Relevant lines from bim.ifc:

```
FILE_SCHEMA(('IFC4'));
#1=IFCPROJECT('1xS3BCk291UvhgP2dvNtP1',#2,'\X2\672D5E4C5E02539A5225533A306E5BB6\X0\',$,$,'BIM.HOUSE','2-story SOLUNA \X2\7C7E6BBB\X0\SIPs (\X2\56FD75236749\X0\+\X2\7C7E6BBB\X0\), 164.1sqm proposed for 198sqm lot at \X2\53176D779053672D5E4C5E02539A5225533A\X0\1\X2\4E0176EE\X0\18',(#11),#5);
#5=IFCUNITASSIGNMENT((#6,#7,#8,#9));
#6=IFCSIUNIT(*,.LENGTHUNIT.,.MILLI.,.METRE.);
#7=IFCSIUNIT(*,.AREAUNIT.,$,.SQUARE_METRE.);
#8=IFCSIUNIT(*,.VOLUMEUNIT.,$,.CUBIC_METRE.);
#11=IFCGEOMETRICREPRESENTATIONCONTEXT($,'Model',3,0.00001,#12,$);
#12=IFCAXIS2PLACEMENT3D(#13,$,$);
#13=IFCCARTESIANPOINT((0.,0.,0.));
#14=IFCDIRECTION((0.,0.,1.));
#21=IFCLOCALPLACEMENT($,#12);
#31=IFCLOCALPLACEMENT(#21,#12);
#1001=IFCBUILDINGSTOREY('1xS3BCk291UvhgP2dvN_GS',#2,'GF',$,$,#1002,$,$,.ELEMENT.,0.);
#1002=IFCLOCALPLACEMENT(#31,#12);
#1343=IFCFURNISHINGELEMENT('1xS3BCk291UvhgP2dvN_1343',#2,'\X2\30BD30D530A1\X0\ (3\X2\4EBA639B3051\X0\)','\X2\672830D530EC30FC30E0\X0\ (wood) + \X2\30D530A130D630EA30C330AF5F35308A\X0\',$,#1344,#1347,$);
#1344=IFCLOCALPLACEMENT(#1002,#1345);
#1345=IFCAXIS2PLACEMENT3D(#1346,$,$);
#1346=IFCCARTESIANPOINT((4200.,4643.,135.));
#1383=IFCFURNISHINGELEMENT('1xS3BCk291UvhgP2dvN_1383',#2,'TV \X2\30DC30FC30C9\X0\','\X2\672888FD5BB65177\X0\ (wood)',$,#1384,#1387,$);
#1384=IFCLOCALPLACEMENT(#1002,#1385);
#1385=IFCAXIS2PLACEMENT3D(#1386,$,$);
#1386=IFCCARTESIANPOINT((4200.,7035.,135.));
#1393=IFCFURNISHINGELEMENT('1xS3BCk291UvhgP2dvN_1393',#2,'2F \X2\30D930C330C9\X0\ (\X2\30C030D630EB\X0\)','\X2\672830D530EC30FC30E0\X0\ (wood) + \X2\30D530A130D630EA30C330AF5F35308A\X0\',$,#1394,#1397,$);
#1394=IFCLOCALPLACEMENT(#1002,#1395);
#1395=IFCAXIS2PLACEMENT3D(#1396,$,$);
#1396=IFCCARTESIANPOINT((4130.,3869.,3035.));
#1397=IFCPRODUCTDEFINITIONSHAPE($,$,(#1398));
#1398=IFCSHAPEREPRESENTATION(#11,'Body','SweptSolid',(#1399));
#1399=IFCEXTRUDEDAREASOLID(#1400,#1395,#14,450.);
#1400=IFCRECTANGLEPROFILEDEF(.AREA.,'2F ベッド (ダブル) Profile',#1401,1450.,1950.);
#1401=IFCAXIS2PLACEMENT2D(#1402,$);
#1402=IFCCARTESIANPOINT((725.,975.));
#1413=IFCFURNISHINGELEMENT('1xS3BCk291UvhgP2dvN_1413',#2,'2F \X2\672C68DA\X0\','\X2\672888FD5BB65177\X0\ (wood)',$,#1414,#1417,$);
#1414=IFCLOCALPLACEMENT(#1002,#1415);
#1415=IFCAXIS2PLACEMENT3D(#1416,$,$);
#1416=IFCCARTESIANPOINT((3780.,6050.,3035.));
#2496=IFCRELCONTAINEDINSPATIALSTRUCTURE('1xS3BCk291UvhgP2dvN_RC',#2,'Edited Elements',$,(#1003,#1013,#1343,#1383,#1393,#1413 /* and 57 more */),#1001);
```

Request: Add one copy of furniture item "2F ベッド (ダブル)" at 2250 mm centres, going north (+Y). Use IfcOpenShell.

```python
import numpy as np
import ifcopenshell
import ifcopenshell.api.geometry
import ifcopenshell.api.root
import ifcopenshell.util.element
import ifcopenshell.util.placement
import ifcopenshell.util.unit

model = ifcopenshell.open("bim.ifc")
unit_scale = ifcopenshell.util.unit.calculate_unit_scale(model)


def reuse_history(source, copy):
    """copy_class also copies each property set's owner history, people and application; keep the originals."""
    for rel in copy.IsDefinedBy:
        if rel.is_a("IfcRelDefinesByProperties") and (history := rel.RelatingPropertyDefinition.OwnerHistory):
            rel.RelatingPropertyDefinition.OwnerHistory = source.OwnerHistory
            ifcopenshell.util.element.remove_deep2(model, history)


source = model.by_id(1393)
base = ifcopenshell.util.placement.get_local_placement(source.ObjectPlacement)
step = np.array([0.0, 1.0, 0.0]) * 2.25 / unit_scale

for i in range(1, 2):
    copy = ifcopenshell.api.root.copy_class(model, product=source)
    copy.Representation = ifcopenshell.util.element.copy_deep(
        model, source.Representation, exclude=["IfcGeometricRepresentationContext", "IfcRepresentationMap"]
    )
    reuse_history(source, copy)
    matrix = base.copy()
    matrix[:3, 3] += i * step
    print("added at", matrix[:3, 3].round(3) + 0.0)
    ifcopenshell.api.geometry.edit_object_placement(model, product=copy, matrix=matrix, is_si=False)

model.write("bim_v2.ifc")
```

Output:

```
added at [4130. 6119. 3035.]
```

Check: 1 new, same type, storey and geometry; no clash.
